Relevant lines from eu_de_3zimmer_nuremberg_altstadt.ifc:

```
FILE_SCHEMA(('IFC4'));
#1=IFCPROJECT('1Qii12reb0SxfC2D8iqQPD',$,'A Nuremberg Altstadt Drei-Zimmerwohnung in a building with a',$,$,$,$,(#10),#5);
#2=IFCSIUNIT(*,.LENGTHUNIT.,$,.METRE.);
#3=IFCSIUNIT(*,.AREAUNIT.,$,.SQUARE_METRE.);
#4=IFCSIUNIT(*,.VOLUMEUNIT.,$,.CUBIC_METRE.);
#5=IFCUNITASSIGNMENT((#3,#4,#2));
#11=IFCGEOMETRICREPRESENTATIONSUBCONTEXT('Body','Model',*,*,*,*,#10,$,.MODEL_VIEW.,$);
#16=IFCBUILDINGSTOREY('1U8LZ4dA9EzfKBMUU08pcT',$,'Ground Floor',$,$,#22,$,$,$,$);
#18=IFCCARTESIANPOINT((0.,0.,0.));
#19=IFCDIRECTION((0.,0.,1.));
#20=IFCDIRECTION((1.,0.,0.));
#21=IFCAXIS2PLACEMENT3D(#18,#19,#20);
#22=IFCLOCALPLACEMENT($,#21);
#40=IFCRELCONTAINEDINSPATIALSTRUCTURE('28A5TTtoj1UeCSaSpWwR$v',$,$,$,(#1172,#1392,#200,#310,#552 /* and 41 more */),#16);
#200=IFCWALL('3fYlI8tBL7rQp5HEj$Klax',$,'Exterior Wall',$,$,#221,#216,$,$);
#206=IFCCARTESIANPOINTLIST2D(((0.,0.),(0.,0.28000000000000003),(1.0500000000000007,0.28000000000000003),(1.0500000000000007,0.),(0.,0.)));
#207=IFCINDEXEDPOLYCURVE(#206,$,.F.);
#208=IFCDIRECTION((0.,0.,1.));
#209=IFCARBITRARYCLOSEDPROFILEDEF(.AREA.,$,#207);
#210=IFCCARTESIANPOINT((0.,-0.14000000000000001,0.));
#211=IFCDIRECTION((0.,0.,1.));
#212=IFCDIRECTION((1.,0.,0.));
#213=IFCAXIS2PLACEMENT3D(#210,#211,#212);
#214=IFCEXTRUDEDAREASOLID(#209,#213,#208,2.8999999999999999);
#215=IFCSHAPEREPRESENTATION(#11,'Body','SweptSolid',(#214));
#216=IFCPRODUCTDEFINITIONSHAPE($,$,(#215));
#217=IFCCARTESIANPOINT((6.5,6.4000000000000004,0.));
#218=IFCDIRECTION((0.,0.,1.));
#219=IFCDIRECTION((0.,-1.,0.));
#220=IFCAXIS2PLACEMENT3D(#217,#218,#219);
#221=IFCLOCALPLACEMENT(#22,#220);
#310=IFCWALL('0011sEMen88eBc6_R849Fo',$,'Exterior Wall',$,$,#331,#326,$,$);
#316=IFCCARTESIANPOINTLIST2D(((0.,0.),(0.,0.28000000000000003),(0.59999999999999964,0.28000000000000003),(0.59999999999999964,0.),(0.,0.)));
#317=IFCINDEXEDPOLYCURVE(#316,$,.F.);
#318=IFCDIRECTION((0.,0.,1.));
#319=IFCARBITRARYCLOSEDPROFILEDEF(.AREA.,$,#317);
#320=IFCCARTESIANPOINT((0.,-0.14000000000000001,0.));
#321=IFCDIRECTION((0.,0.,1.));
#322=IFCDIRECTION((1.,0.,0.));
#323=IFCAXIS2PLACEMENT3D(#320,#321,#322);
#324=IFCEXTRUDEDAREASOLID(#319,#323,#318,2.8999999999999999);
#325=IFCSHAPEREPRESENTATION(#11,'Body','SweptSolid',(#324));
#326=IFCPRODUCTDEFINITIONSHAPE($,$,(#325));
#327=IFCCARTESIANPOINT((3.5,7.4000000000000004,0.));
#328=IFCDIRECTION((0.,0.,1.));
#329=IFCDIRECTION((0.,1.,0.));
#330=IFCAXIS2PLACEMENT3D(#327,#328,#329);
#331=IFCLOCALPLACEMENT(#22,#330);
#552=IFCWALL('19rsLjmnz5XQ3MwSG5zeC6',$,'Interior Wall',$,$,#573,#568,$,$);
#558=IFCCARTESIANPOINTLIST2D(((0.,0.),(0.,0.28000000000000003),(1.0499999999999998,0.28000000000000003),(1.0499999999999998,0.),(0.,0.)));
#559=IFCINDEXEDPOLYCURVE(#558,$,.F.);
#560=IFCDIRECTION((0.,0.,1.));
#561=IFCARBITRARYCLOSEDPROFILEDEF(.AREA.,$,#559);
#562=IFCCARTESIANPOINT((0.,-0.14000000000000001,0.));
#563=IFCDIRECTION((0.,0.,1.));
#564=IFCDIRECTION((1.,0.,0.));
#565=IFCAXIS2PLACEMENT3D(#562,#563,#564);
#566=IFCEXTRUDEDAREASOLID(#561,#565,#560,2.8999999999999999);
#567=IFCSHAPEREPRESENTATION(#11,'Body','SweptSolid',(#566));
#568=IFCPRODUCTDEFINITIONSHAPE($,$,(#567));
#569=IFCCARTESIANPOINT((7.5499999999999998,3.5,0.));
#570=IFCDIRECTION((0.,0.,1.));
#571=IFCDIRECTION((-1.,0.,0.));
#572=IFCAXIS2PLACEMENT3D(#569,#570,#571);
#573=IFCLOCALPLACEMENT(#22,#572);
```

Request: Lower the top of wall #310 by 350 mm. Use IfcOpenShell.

```python
import ifcopenshell
import ifcopenshell.geom
import ifcopenshell.util.representation
import ifcopenshell.util.shape

model = ifcopenshell.open("eu_de_3zimmer_nuremberg_altstadt.ifc")
settings = ifcopenshell.geom.settings()


def volume(element):
    """Net volume in cubic metres, openings subtracted."""
    shape = ifcopenshell.geom.create_shape(settings, element)
    return ifcopenshell.util.shape.get_volume(shape.geometry)


wall = model.by_guid("0011sEMen88eBc6_R849Fo")
before = volume(wall)

body = ifcopenshell.util.representation.get_representation(wall, "Model", "Body")
solid = body.Items[0]
old_height = solid.Depth
solid.Depth -= 0.35
after = volume(wall)

print(f"height {old_height:g} -> {solid.Depth:g}, volume {before:.3f} -> {after:.3f} m3")

model.write("eu_de_3zimmer_nuremberg_altstadt_rev.ifc")
```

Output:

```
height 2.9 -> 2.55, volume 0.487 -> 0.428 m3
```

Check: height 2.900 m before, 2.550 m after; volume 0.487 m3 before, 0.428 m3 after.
